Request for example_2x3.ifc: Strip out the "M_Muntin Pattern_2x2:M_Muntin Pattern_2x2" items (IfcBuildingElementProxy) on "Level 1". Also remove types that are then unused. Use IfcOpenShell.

First a look at what the model holds.

```python
import ifcopenshell
import ifcopenshell.util.element

model = ifcopenshell.open("example_2x3.ifc")
print(model.schema)
storey = next(s for s in model.by_type("IfcBuildingStorey") if s.Name == "Level 1")
proxies = [e for e in ifcopenshell.util.element.get_decomposition(storey) if e.is_a("IfcBuildingElementProxy")]
seen = {}
for e in proxies:
    element_type = ifcopenshell.util.element.get_type(e)
    name = element_type.Name if element_type not in (None, e) else None
    seen[name] = seen.get(name, 0) + 1
for name, count in sorted(seen.items(), key=str):
    print(count, "x", name)
```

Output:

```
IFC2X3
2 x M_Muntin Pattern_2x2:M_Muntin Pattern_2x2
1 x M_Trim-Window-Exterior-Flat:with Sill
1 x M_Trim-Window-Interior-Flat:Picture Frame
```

```python
import ifcopenshell
import ifcopenshell.api.root
import ifcopenshell.util.element

model = ifcopenshell.open("example_2x3.ifc")

storey = next(s for s in model.by_type("IfcBuildingStorey") if s.Name == "Level 1")
proxies = [e for e in ifcopenshell.util.element.get_decomposition(storey) if e.is_a("IfcBuildingElementProxy")]
targets = [e for e in proxies if (t := ifcopenshell.util.element.get_type(e)) not in (None, e) and t.Name == "M_Muntin Pattern_2x2:M_Muntin Pattern_2x2"]
types = {ifcopenshell.util.element.get_type(e) for e in targets} - {None, *targets}

for e in targets:
    ifcopenshell.api.root.remove_product(model, product=e)
print(len(targets), "removed")

unused = [t for t in types if not ifcopenshell.util.element.get_types(t)]
for t in unused:
    ifcopenshell.api.root.remove_product(model, product=t)
print(len(unused), "unused types removed")

model.write("example_2x3_updated.ifc")
```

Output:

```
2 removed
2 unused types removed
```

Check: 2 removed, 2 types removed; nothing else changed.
